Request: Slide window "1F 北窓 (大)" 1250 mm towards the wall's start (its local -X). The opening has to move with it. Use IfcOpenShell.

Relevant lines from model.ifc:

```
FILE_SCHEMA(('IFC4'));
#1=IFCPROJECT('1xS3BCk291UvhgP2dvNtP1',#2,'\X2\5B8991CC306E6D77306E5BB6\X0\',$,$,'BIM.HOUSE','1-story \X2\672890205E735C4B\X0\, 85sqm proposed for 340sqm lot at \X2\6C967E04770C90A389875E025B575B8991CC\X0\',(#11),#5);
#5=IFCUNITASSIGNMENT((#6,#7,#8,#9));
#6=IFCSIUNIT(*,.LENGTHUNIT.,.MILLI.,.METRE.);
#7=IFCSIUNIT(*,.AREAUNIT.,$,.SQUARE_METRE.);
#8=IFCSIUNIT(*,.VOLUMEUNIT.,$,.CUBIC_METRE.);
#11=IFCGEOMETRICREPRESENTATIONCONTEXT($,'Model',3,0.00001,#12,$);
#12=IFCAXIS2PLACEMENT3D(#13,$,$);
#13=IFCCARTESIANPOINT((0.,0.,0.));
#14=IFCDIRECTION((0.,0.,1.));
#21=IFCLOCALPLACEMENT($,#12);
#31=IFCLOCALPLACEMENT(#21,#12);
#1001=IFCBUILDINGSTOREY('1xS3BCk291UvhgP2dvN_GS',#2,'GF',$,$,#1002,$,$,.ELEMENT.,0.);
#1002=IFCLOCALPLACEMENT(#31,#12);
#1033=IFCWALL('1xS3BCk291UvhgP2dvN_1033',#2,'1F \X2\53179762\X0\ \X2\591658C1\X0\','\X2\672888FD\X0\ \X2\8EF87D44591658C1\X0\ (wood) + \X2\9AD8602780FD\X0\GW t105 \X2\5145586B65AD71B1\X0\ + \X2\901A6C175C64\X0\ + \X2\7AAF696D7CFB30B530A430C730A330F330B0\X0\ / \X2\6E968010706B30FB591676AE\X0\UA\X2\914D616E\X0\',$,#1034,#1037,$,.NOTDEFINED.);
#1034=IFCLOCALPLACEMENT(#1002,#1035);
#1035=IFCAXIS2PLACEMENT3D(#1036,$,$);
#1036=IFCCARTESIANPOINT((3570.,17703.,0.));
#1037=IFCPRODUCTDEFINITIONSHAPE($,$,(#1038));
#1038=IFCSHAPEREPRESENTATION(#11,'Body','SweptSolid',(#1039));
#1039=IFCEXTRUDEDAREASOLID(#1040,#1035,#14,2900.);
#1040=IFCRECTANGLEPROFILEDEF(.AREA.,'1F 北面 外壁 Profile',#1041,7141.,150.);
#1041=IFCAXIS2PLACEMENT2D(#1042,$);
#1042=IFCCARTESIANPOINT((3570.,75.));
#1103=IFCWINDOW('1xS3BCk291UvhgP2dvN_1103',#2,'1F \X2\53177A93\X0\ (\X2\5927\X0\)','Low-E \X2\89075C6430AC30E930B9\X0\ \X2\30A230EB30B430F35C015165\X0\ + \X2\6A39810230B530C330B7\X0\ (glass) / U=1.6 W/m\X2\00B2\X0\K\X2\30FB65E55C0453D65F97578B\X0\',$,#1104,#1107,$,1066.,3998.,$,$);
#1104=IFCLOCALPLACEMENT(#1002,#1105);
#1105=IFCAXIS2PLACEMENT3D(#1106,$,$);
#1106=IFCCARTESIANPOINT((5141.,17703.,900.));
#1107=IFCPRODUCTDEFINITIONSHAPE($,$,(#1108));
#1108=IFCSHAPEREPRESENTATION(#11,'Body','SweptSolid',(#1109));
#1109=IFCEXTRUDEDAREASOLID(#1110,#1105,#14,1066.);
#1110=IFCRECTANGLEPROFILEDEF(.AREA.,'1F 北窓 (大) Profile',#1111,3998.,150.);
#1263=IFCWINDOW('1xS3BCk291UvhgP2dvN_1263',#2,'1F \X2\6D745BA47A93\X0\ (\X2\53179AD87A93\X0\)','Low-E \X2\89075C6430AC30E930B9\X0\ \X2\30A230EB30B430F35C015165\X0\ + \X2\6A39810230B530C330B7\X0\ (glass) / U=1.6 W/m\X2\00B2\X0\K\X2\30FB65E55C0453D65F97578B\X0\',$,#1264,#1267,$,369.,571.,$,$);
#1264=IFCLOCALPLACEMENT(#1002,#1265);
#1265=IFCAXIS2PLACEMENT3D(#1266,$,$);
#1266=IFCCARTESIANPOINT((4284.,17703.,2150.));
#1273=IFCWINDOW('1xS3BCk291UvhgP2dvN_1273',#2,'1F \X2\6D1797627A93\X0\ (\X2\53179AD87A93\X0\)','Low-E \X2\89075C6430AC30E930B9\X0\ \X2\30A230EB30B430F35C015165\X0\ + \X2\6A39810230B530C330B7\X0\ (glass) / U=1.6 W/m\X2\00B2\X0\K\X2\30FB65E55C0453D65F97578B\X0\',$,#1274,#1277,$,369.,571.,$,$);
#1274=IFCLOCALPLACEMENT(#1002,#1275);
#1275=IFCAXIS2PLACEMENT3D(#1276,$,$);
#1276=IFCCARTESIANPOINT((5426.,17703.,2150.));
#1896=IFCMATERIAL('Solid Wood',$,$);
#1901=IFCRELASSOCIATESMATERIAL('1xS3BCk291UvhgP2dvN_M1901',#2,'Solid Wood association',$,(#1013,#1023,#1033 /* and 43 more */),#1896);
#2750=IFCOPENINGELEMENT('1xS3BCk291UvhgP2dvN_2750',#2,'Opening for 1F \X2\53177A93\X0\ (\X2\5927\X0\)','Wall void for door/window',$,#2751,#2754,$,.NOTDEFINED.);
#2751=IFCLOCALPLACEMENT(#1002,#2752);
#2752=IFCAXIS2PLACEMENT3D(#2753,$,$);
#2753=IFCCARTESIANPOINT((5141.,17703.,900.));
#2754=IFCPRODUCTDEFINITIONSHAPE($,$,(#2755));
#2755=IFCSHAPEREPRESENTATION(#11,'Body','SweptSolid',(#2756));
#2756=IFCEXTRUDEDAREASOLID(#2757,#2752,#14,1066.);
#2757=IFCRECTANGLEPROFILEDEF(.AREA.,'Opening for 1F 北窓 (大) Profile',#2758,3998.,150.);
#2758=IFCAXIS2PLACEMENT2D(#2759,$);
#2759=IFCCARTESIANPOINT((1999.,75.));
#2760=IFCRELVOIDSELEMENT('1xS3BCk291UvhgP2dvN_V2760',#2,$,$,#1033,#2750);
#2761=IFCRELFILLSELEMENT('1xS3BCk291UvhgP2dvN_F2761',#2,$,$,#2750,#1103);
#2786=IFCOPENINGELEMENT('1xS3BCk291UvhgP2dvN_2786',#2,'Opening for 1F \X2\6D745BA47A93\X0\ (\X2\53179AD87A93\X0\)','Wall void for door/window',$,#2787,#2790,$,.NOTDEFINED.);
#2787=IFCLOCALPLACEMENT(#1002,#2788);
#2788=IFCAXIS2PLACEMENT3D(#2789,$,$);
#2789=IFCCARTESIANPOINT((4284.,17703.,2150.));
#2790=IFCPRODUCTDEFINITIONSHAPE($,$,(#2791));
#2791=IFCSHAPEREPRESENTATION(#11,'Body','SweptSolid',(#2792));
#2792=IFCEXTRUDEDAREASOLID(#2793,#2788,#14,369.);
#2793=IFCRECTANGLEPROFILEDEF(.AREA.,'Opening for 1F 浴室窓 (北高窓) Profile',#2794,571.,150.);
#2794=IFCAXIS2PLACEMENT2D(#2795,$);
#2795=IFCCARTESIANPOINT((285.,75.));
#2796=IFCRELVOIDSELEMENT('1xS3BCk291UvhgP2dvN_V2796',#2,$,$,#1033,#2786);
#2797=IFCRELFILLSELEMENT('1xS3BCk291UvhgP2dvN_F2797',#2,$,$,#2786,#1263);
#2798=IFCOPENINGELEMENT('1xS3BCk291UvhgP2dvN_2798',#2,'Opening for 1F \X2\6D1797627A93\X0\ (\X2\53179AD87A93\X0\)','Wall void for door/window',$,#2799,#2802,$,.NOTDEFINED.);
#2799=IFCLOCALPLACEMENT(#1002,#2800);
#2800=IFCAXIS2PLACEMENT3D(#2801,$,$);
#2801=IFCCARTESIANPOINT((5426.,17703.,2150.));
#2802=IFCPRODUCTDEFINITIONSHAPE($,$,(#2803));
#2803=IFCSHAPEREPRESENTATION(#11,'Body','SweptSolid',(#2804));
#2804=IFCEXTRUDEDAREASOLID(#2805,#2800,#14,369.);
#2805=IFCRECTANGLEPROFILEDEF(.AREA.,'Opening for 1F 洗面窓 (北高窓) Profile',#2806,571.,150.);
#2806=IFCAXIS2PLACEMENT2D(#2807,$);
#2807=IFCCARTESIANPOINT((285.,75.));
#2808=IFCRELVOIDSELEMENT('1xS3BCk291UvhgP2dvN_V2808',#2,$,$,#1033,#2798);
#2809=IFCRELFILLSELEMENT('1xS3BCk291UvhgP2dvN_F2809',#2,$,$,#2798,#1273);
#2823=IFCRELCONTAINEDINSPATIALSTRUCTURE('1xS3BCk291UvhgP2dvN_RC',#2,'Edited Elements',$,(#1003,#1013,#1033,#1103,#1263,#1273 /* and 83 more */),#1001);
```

```python
import ifcopenshell
import ifcopenshell.api.geometry
import ifcopenshell.util.placement
import ifcopenshell.util.unit

model = ifcopenshell.open("model.ifc")
unit_scale = ifcopenshell.util.unit.calculate_unit_scale(model)

window = model.by_id(1103)
opening = window.FillsVoids[0].RelatingOpeningElement
wall = opening.VoidsElements[0].RelatingBuildingElement

wall_matrix = ifcopenshell.util.placement.get_local_placement(wall.ObjectPlacement)
shift = wall_matrix[:3, 0] * -1.25 / unit_scale
before = ifcopenshell.util.placement.get_local_placement(window.ObjectPlacement)[:3, 3].copy()

# The window is not placed relative to its opening, so move both.
for product in (opening, window):
    matrix = ifcopenshell.util.placement.get_local_placement(product.ObjectPlacement)
    matrix[:3, 3] += shift
    ifcopenshell.api.geometry.edit_object_placement(model, product=product, matrix=matrix, is_si=False)

after = ifcopenshell.util.placement.get_local_placement(window.ObjectPlacement)[:3, 3]
print("window moved by", (after - before).round(3) + 0.0)

model.write("model_updated.ifc")
```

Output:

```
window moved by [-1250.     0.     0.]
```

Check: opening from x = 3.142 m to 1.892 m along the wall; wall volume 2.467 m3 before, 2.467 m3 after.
